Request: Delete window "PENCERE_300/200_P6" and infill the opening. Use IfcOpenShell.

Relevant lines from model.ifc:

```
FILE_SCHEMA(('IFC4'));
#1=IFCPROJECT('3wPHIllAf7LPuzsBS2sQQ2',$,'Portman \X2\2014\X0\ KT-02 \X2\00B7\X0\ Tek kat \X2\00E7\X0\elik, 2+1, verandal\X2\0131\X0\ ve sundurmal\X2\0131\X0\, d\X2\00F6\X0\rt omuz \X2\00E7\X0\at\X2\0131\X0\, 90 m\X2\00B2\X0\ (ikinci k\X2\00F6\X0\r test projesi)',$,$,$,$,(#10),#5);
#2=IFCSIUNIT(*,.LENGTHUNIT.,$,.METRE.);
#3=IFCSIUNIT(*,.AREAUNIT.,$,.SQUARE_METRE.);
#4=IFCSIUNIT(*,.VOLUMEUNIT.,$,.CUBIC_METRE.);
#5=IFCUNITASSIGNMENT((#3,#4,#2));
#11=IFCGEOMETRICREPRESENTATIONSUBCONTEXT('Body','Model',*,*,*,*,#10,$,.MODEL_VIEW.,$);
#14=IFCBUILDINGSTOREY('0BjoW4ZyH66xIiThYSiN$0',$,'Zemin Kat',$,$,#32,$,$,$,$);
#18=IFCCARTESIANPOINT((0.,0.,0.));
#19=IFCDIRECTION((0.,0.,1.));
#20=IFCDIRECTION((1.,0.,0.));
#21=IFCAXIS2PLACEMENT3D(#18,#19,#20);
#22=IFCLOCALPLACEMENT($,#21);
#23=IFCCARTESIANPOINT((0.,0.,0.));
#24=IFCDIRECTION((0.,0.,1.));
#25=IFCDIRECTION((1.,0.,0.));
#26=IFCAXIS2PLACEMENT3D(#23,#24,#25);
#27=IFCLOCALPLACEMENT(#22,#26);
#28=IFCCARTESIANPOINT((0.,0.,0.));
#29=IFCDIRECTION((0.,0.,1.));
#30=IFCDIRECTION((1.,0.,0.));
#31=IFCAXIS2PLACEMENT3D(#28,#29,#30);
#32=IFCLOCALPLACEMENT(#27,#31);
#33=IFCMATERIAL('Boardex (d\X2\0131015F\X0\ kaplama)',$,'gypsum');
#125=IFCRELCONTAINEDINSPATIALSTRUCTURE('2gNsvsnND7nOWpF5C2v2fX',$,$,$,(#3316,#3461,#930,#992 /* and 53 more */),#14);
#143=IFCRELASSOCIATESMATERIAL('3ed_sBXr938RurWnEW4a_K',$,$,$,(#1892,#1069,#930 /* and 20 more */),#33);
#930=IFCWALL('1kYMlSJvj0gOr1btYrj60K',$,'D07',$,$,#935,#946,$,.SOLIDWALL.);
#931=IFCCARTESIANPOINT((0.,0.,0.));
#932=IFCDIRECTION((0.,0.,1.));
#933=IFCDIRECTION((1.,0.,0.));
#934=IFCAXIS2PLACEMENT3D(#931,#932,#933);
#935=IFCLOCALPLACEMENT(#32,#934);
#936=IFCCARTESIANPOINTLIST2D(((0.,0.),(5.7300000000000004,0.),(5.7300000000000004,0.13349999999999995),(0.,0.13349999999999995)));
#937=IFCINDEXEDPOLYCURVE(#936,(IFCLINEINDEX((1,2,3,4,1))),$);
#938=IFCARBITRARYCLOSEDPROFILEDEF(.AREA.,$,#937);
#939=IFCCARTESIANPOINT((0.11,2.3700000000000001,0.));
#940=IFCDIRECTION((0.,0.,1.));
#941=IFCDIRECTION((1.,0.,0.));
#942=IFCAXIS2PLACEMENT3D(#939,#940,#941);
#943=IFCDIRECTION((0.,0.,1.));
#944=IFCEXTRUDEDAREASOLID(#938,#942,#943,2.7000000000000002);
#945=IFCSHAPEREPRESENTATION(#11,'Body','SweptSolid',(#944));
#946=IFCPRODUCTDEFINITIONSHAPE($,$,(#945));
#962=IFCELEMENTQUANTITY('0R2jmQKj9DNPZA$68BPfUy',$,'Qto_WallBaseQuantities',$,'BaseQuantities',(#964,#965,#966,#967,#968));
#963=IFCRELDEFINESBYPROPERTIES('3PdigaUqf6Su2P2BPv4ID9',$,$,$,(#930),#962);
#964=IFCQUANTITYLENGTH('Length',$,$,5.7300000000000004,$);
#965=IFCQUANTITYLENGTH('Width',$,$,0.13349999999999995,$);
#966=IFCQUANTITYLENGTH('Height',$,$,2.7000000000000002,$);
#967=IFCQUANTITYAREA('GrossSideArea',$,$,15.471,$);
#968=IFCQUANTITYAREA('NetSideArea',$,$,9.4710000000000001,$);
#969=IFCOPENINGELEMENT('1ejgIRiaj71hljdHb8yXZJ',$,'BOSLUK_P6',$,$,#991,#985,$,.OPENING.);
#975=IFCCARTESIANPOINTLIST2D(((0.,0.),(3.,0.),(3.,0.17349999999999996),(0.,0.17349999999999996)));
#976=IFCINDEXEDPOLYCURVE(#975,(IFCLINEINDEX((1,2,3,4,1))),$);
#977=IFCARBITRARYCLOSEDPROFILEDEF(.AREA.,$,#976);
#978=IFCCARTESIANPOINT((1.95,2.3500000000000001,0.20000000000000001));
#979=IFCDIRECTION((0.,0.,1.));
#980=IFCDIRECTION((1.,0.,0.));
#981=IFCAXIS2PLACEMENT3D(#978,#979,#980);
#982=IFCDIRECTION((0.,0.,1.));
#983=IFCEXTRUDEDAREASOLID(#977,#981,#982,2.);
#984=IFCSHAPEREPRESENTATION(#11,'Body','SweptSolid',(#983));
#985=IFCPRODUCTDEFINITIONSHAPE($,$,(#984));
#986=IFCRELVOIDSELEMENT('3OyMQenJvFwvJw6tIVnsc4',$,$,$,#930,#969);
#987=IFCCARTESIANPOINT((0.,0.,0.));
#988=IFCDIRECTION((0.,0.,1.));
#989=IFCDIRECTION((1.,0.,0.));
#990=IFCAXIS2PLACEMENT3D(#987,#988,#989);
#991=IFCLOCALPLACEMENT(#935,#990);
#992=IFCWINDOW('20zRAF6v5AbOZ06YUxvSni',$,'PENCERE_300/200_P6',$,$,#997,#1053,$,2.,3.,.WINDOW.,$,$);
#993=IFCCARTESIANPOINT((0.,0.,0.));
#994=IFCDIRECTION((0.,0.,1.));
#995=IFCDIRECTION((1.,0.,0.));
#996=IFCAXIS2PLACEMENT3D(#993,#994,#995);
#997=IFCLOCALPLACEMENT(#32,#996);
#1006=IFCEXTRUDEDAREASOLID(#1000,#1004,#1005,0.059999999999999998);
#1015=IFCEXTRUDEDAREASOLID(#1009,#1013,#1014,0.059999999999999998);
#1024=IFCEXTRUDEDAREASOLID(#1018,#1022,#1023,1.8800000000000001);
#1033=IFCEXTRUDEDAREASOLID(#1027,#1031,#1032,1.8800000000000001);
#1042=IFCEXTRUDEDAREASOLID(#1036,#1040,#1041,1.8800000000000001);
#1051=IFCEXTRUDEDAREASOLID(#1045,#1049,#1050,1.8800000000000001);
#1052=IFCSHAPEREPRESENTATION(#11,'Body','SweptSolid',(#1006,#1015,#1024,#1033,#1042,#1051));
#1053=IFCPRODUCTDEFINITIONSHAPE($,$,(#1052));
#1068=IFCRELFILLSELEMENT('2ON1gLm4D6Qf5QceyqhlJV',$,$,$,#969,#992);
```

```python
import ifcopenshell
import ifcopenshell.api.feature
import ifcopenshell.api.pset
import ifcopenshell.api.root
import ifcopenshell.geom
import ifcopenshell.util.element
import ifcopenshell.util.shape
import ifcopenshell.util.unit

model = ifcopenshell.open("model.ifc")
area_scale = ifcopenshell.util.unit.calculate_unit_scale(model, "AREAUNIT")
settings = ifcopenshell.geom.settings()


def volume(element):
    """Net volume in cubic metres, openings subtracted."""
    shape = ifcopenshell.geom.create_shape(settings, element)
    return ifcopenshell.util.shape.get_volume(shape.geometry)


window = model.by_guid("20zRAF6v5AbOZ06YUxvSni")
opening = window.FillsVoids[0].RelatingOpeningElement
wall = opening.VoidsElements[0].RelatingBuildingElement
before = volume(wall)

ifcopenshell.api.root.remove_product(model, product=window)
ifcopenshell.api.feature.remove_feature(model, feature=opening)

after = volume(wall)
thickness = 0.1335  # wall thickness in metres

# Update the wall's stored quantities.
qto = model.by_id(ifcopenshell.util.element.get_pset(wall, "Qto_WallBaseQuantities", should_inherit=False)["id"])
ifcopenshell.api.pset.edit_qto(model, qto=qto, properties={"NetSideArea": after / thickness / area_scale})

print(f"wall volume {before:.3f} -> {after:.3f} m3")

model.write("model_edited.ifc")
```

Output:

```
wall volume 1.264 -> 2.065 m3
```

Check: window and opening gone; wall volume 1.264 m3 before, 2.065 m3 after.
